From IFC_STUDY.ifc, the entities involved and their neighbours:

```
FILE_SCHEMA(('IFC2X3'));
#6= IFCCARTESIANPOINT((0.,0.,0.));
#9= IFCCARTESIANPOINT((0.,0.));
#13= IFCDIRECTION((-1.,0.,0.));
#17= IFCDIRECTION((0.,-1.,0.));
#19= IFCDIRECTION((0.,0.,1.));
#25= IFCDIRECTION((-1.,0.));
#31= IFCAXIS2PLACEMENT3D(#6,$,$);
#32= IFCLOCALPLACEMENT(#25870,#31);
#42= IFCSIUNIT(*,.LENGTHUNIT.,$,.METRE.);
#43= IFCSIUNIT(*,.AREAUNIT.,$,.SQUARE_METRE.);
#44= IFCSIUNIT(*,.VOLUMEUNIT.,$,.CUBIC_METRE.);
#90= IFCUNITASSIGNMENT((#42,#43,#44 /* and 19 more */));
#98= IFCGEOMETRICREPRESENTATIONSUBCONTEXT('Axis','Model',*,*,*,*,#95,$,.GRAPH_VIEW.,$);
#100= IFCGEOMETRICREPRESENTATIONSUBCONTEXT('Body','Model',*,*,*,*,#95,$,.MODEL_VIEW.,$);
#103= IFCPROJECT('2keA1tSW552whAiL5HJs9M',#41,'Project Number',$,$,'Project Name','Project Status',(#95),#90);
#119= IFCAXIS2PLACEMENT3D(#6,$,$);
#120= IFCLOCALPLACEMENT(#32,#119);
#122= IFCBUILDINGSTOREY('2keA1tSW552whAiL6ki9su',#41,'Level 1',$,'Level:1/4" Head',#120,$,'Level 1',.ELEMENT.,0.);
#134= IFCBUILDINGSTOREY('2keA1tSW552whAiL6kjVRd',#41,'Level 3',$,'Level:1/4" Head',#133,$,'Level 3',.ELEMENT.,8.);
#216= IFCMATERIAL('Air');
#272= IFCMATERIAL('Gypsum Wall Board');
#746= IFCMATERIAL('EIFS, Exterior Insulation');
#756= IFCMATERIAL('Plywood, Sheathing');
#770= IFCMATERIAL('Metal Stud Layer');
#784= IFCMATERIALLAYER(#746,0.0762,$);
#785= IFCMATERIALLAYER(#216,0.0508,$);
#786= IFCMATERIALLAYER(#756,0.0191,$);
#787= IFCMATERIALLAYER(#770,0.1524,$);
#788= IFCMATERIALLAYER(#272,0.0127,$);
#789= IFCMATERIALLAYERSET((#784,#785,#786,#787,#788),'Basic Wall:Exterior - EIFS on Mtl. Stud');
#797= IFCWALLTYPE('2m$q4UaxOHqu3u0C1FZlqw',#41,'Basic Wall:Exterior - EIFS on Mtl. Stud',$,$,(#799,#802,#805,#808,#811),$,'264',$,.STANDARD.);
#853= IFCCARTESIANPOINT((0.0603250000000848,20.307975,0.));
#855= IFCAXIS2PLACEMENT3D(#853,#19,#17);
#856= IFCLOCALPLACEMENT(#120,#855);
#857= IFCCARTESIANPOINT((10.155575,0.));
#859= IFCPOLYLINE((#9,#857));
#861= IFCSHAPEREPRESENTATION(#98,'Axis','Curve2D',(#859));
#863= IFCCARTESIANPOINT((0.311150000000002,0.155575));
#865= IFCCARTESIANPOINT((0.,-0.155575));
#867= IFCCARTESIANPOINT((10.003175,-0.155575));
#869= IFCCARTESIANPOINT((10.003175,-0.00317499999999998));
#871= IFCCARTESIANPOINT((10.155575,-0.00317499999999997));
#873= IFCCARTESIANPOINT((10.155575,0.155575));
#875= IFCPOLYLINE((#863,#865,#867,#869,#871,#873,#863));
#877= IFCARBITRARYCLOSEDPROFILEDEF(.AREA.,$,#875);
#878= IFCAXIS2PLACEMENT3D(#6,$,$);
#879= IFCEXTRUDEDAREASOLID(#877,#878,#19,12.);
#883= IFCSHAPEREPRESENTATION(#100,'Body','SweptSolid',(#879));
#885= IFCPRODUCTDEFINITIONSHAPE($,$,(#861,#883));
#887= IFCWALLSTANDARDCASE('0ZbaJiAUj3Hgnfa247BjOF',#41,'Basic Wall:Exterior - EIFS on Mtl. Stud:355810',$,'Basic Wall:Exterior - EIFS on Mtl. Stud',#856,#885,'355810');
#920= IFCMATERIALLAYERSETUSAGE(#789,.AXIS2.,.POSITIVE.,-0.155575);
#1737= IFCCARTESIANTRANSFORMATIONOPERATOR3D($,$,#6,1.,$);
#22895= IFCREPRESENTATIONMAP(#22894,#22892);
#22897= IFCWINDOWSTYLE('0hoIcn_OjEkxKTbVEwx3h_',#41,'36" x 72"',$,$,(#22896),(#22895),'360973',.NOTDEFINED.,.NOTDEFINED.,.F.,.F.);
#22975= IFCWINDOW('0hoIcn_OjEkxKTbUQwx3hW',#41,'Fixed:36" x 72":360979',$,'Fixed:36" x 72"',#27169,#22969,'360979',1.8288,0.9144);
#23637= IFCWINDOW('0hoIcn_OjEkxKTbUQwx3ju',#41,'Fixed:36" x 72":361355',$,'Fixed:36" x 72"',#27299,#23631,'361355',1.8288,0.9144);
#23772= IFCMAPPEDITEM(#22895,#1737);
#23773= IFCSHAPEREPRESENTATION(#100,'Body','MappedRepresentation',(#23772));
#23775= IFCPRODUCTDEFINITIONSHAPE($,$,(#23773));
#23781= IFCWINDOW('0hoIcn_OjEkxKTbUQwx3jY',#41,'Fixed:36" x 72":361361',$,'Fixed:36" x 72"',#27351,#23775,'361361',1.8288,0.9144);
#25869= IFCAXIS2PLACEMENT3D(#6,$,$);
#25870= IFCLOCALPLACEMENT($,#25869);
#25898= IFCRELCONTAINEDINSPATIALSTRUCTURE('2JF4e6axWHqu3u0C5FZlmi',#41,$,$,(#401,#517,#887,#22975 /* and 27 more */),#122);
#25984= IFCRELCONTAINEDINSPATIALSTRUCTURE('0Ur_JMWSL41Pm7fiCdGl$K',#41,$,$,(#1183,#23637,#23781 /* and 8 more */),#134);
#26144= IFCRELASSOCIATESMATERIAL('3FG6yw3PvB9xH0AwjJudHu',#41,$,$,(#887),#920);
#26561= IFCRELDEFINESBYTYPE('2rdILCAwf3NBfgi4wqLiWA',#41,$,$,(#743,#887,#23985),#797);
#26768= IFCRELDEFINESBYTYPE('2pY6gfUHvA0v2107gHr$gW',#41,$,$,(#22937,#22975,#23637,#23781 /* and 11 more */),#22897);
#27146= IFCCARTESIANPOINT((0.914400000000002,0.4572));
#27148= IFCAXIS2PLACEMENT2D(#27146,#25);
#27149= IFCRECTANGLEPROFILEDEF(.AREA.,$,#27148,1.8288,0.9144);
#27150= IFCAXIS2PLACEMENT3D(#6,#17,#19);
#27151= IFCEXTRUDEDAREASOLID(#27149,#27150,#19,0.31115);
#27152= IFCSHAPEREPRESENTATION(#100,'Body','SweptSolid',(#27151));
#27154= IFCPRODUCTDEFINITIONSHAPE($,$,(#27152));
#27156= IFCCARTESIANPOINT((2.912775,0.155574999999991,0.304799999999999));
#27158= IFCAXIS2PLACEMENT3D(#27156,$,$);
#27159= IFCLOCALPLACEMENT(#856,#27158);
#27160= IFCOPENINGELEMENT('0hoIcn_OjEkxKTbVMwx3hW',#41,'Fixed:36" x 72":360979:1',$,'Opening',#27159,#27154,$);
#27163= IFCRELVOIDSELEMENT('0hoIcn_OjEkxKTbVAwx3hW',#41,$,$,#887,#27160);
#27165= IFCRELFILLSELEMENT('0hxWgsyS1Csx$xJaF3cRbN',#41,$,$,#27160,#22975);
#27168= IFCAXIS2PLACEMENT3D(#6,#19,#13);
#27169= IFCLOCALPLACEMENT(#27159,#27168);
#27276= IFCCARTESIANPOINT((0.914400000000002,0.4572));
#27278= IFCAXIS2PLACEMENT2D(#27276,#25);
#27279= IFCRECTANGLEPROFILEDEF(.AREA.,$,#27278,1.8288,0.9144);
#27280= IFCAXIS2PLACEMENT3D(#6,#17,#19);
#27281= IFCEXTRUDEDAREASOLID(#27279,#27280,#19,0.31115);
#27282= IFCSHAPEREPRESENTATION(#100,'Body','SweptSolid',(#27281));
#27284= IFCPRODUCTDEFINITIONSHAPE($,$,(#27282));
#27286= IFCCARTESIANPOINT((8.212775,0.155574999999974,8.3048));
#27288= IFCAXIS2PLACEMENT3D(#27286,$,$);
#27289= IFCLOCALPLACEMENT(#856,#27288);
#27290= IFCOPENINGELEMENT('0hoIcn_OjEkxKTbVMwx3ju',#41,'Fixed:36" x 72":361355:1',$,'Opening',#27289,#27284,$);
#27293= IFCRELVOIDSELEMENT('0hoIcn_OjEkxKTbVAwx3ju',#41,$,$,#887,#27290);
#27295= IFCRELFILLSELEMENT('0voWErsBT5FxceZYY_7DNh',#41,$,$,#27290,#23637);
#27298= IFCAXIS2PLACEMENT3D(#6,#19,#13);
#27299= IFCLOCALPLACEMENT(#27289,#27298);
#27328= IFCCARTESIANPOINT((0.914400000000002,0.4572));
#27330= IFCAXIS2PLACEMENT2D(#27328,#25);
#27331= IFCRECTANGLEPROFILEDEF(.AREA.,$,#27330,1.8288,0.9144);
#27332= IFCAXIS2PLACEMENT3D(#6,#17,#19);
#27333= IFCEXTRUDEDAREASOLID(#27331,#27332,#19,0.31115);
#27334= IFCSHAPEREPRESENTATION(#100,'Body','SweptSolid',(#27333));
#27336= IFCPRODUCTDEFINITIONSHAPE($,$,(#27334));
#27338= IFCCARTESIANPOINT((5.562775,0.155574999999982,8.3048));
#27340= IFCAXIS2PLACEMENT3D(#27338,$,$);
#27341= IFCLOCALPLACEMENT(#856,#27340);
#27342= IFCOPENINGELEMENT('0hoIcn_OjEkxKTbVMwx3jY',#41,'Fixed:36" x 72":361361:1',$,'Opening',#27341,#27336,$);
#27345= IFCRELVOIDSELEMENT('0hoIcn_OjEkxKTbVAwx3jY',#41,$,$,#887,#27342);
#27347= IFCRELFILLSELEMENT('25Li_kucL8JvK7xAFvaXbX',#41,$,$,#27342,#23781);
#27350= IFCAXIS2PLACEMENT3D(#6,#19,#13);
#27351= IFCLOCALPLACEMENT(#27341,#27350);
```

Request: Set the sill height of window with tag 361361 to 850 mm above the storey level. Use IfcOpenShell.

```python
import numpy as np
import ifcopenshell
import ifcopenshell.api.geometry
import ifcopenshell.geom
import ifcopenshell.util.element
import ifcopenshell.util.placement
import ifcopenshell.util.shape
import ifcopenshell.util.unit

model = ifcopenshell.open("IFC_STUDY.ifc")
unit_scale = ifcopenshell.util.unit.calculate_unit_scale(model)

window = model.by_guid("0hoIcn_OjEkxKTbUQwx3jY")
opening = window.FillsVoids[0].RelatingOpeningElement
storey = ifcopenshell.util.element.get_container(window, ifc_class="IfcBuildingStorey")
level = ifcopenshell.util.placement.get_local_placement(storey.ObjectPlacement)[2, 3]

# The opening's origin need not be at the sill, so measure its lowest point.
shape = ifcopenshell.geom.create_shape(ifcopenshell.geom.settings(), opening)
bottom = ifcopenshell.util.shape.get_shape_bottom_elevation(shape, shape.geometry) / unit_scale
dz = level + 0.85 / unit_scale - bottom

shift = np.array([0.0, 0.0, dz])
# The window is placed relative to its opening, so it follows when the opening moves.
matrix = ifcopenshell.util.placement.get_local_placement(opening.ObjectPlacement)
matrix[:3, 3] += shift
ifcopenshell.api.geometry.edit_object_placement(
    model, product=opening, matrix=matrix, is_si=False, should_transform_children=True
)

print(f"moved by {dz * unit_scale:+.3f} m")

model.write("IFC_STUDY_v2.ifc")
```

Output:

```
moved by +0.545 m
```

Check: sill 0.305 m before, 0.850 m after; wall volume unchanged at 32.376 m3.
